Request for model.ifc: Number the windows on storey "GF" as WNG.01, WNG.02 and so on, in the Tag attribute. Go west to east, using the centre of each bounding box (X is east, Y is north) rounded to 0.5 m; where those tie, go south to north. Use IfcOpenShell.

First a look at what the model holds.

```python
import ifcopenshell
import ifcopenshell.util.element
import ifcopenshell.util.placement

model = ifcopenshell.open("model.ifc")
print(model.schema)
storey = next(s for s in model.by_type("IfcBuildingStorey") if s.Name == "GF")
windows = [e for e in ifcopenshell.util.element.get_decomposition(storey) if e.is_a("IfcWindow")]
for e in sorted(windows, key=lambda e: e.id()):
    origin = ifcopenshell.util.placement.get_local_placement(e.ObjectPlacement)[:3, 3]
    print(e.id(), e.Tag, e.Name, origin.round(2) + 0.0, sep=" | ")
```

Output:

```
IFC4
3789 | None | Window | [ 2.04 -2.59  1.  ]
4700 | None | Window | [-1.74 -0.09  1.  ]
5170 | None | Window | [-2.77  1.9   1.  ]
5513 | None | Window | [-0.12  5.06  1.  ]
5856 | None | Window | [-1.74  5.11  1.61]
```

```python
import ifcopenshell
import ifcopenshell.geom
import ifcopenshell.util.element
import ifcopenshell.util.shape

model = ifcopenshell.open("model.ifc")
settings = ifcopenshell.geom.settings()
settings.set("use-world-coords", True)


def centre(element):
    shape = ifcopenshell.geom.create_shape(settings, element)
    return ifcopenshell.util.shape.get_bbox_centroid(shape.geometry)


storey = next(s for s in model.by_type("IfcBuildingStorey") if s.Name == "GF")
windows = [e for e in ifcopenshell.util.element.get_decomposition(storey) if e.is_a("IfcWindow")]

# Insertion points can sit at a corner or the storey origin, so sort by the geometry (in metres).
centres = {e: centre(e) for e in windows}
windows.sort(key=lambda e: (round(centres[e][0] / 0.5), centres[e][1]))

for i, e in enumerate(windows, start=1):
    number = f"WNG.{i:02d}"
    e.Tag = number
    print(e.id(), number)

model.write("model_rev.ifc")
```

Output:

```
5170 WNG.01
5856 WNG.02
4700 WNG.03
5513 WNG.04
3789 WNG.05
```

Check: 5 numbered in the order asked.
